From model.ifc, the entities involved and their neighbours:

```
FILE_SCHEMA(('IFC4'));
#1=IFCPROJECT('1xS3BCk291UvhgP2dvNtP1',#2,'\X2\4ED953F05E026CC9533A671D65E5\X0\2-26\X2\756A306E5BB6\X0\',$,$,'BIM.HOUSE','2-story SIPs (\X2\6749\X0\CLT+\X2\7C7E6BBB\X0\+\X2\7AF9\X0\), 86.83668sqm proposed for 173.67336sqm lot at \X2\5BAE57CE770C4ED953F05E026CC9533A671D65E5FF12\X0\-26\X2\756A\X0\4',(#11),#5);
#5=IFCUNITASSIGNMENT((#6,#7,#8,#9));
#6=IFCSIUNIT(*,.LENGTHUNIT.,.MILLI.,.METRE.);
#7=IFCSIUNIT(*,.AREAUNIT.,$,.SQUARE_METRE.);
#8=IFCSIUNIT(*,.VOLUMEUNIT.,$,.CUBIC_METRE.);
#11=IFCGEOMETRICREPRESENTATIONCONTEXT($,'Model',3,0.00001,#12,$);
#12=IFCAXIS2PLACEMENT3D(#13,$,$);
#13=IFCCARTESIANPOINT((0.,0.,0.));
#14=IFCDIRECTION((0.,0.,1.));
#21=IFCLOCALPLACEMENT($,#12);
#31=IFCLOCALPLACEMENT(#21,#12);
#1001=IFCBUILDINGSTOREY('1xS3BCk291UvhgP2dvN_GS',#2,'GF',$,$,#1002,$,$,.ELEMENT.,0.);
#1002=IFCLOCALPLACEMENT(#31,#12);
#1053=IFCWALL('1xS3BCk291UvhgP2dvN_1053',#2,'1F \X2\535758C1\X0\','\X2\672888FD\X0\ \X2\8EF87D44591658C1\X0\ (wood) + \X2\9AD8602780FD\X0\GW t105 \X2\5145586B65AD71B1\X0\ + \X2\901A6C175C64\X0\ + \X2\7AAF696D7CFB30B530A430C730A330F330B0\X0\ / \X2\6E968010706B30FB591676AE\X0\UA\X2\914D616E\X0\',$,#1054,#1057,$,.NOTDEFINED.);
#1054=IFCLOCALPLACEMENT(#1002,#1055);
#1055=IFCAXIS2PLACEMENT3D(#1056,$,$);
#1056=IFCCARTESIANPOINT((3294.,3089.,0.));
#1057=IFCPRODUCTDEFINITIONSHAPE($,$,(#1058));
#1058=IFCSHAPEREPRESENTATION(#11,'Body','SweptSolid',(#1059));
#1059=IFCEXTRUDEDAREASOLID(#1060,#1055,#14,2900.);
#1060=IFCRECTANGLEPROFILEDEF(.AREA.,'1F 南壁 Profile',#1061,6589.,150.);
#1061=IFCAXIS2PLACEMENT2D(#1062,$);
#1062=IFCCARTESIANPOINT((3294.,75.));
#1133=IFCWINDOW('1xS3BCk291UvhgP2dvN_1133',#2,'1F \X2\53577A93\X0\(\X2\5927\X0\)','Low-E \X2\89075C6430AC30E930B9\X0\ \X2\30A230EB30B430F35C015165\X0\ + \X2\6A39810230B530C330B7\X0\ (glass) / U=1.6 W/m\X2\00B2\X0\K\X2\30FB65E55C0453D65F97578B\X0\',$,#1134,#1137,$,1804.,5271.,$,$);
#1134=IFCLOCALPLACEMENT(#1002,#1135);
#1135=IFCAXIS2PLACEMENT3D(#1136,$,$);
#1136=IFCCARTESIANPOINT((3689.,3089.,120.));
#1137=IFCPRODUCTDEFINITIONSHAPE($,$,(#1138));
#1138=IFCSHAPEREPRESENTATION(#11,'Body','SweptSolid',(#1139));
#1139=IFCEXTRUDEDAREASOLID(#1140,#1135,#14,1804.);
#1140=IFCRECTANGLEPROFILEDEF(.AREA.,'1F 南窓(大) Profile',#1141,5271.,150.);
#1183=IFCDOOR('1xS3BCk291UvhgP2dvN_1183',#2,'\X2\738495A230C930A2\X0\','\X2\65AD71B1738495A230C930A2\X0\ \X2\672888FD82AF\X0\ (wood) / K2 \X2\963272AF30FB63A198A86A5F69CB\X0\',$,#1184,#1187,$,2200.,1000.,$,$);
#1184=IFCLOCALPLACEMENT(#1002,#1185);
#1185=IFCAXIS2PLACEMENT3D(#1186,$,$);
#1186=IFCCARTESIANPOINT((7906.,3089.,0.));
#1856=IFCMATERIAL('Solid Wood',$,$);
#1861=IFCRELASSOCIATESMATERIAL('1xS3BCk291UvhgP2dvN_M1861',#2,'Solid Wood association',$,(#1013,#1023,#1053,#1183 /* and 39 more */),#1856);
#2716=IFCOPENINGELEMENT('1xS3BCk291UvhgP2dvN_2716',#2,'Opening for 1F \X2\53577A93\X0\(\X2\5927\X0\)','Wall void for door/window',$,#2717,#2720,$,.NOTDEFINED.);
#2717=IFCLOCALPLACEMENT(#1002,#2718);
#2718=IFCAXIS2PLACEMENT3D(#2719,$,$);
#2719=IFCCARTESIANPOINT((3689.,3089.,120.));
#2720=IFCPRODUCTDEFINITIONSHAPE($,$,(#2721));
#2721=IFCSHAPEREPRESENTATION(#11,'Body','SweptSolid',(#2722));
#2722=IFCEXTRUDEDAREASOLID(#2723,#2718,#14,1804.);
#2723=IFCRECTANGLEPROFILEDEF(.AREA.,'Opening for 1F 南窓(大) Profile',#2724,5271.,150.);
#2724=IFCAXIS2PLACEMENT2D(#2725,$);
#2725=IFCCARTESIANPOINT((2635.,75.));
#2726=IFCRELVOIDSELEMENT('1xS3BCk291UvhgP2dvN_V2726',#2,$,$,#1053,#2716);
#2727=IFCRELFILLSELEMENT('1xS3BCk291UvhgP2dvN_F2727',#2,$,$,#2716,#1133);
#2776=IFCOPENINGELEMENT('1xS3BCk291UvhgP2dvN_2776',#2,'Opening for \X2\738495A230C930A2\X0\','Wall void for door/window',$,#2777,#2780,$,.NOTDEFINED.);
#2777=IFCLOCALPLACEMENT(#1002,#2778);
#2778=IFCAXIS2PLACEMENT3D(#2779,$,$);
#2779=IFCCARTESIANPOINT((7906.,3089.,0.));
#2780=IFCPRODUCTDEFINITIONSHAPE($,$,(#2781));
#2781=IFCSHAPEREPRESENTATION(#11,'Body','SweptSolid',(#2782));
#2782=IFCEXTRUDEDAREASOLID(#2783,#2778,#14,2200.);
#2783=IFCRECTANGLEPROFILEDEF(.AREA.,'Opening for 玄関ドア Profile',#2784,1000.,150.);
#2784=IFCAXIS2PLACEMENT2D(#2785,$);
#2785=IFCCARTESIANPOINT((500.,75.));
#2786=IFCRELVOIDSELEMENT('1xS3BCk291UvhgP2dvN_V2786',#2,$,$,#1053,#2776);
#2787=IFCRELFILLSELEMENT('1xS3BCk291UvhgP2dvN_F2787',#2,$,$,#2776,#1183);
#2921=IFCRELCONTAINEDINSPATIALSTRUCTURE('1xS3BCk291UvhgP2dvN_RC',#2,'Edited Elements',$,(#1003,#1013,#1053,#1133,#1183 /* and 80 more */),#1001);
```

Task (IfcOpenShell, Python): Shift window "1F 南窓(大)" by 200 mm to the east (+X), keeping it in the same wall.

```python
import ifcopenshell
import ifcopenshell.api.geometry
import ifcopenshell.util.placement
import ifcopenshell.util.unit

model = ifcopenshell.open("model.ifc")
unit_scale = ifcopenshell.util.unit.calculate_unit_scale(model)

window = model.by_id(1133)
opening = window.FillsVoids[0].RelatingOpeningElement
wall = opening.VoidsElements[0].RelatingBuildingElement

wall_matrix = ifcopenshell.util.placement.get_local_placement(wall.ObjectPlacement)
shift = wall_matrix[:3, 0] * 0.2 / unit_scale
before = ifcopenshell.util.placement.get_local_placement(window.ObjectPlacement)[:3, 3].copy()

# The window is not placed relative to its opening, so move both.
for product in (opening, window):
    matrix = ifcopenshell.util.placement.get_local_placement(product.ObjectPlacement)
    matrix[:3, 3] += shift
    ifcopenshell.api.geometry.edit_object_placement(model, product=product, matrix=matrix, is_si=False)

after = ifcopenshell.util.placement.get_local_placement(window.ObjectPlacement)[:3, 3]
print("window moved by", (after - before).round(3) + 0.0)

model.write("model_updated.ifc")
```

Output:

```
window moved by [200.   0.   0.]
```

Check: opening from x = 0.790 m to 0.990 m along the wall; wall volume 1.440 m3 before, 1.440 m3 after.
